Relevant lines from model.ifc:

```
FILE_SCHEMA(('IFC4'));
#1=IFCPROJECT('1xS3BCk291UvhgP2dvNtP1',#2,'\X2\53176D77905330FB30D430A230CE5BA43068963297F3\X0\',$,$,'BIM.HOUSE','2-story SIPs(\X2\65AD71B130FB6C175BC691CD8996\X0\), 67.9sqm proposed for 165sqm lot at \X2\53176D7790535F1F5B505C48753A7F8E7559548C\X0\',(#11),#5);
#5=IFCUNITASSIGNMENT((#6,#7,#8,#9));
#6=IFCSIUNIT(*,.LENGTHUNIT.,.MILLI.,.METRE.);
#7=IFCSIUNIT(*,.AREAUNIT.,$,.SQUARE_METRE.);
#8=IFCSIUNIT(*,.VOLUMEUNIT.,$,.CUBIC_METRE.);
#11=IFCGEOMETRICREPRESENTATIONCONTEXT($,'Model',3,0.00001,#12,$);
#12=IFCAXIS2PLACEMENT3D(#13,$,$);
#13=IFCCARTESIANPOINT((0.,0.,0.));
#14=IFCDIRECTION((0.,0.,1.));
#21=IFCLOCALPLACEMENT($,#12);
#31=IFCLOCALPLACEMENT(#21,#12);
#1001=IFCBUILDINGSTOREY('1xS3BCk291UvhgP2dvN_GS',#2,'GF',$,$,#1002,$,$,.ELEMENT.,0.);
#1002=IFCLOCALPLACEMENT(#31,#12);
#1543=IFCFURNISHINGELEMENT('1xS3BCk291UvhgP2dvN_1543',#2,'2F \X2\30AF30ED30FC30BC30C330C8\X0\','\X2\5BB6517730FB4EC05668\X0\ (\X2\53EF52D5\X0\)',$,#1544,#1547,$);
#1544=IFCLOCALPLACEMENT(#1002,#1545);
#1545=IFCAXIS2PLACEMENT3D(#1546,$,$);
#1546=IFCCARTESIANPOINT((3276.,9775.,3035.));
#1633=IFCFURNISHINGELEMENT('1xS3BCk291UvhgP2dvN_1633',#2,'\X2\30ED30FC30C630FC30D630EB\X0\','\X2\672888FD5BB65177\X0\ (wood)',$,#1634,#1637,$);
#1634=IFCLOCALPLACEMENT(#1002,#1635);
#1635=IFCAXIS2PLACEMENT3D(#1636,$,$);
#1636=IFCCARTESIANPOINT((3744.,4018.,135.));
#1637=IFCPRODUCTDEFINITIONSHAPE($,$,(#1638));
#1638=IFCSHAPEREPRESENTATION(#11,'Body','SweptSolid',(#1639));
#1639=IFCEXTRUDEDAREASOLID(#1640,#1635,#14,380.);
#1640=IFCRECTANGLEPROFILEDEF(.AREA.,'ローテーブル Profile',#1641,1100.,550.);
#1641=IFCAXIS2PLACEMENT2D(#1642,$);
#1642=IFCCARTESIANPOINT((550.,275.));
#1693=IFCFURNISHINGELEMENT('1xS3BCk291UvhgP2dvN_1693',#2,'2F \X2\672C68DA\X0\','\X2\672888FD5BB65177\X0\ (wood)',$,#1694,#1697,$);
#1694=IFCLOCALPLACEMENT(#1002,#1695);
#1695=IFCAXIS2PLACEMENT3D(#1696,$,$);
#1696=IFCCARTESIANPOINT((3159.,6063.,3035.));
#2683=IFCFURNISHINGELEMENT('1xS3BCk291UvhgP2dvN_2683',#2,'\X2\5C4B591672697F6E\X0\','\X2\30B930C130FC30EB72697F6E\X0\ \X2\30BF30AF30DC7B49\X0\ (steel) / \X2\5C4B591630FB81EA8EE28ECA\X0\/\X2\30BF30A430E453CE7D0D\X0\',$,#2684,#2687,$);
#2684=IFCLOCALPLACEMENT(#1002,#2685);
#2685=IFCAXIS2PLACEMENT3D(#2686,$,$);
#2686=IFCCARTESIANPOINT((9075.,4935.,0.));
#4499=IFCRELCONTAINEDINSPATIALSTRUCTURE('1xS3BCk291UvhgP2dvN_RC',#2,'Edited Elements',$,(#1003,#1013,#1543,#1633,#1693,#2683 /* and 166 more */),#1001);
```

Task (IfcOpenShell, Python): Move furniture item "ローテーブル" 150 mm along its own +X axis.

```python
import ifcopenshell
import ifcopenshell.api.geometry
import ifcopenshell.util.placement
import ifcopenshell.util.unit

model = ifcopenshell.open("model.ifc")
unit_scale = ifcopenshell.util.unit.calculate_unit_scale(model)

item = model.by_guid("1xS3BCk291UvhgP2dvN_1633")
matrix = ifcopenshell.util.placement.get_local_placement(item.ObjectPlacement)
matrix[:3, 3] += matrix[:3, 0] * 0.15 / unit_scale
ifcopenshell.api.geometry.edit_object_placement(model, product=item, matrix=matrix, is_si=False)

print(ifcopenshell.util.placement.get_local_placement(item.ObjectPlacement).round(3) + 0.0)

model.write("model_rev.ifc")
```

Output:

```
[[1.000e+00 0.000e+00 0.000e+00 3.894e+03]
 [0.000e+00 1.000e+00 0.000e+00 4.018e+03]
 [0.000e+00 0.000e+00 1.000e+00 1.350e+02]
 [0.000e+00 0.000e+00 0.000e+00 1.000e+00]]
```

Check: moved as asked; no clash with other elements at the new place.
